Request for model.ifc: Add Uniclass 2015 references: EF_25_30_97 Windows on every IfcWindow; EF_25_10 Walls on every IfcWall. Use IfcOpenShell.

First a look at what the model holds.

```python
import ifcopenshell

model = ifcopenshell.open("model.ifc")
print(model.schema)
print("classifications:", [c.Name for c in model.by_type("IfcClassification")])
for ifc_class in ("IfcDoor", "IfcRoof", "IfcStair", "IfcWall", "IfcWindow"):
    print(ifc_class, len(model.by_type(ifc_class)))
```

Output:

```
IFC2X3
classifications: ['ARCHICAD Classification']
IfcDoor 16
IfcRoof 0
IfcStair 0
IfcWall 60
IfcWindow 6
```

```python
import ifcopenshell
import ifcopenshell.api.classification

model = ifcopenshell.open("model.ifc")

# IFC2X3 requires Source and Edition and has no link from the project to the system.
system = model.create_entity("IfcClassification", Source="NBS", Edition="2015", Name="Uniclass 2015")

codes = {
    "IfcWindow": ("EF_25_30_97", "Windows"),
    "IfcWall": ("EF_25_10", "Walls"),
}
for ifc_class, (code, name) in codes.items():
    products = model.by_type(ifc_class)
    ifcopenshell.api.classification.add_reference(
        model, products=products, classification=system, identification=code, name=name
    )
    print(code, len(products))

model.write("model_edited.ifc")
```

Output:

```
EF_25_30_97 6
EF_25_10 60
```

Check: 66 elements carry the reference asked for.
